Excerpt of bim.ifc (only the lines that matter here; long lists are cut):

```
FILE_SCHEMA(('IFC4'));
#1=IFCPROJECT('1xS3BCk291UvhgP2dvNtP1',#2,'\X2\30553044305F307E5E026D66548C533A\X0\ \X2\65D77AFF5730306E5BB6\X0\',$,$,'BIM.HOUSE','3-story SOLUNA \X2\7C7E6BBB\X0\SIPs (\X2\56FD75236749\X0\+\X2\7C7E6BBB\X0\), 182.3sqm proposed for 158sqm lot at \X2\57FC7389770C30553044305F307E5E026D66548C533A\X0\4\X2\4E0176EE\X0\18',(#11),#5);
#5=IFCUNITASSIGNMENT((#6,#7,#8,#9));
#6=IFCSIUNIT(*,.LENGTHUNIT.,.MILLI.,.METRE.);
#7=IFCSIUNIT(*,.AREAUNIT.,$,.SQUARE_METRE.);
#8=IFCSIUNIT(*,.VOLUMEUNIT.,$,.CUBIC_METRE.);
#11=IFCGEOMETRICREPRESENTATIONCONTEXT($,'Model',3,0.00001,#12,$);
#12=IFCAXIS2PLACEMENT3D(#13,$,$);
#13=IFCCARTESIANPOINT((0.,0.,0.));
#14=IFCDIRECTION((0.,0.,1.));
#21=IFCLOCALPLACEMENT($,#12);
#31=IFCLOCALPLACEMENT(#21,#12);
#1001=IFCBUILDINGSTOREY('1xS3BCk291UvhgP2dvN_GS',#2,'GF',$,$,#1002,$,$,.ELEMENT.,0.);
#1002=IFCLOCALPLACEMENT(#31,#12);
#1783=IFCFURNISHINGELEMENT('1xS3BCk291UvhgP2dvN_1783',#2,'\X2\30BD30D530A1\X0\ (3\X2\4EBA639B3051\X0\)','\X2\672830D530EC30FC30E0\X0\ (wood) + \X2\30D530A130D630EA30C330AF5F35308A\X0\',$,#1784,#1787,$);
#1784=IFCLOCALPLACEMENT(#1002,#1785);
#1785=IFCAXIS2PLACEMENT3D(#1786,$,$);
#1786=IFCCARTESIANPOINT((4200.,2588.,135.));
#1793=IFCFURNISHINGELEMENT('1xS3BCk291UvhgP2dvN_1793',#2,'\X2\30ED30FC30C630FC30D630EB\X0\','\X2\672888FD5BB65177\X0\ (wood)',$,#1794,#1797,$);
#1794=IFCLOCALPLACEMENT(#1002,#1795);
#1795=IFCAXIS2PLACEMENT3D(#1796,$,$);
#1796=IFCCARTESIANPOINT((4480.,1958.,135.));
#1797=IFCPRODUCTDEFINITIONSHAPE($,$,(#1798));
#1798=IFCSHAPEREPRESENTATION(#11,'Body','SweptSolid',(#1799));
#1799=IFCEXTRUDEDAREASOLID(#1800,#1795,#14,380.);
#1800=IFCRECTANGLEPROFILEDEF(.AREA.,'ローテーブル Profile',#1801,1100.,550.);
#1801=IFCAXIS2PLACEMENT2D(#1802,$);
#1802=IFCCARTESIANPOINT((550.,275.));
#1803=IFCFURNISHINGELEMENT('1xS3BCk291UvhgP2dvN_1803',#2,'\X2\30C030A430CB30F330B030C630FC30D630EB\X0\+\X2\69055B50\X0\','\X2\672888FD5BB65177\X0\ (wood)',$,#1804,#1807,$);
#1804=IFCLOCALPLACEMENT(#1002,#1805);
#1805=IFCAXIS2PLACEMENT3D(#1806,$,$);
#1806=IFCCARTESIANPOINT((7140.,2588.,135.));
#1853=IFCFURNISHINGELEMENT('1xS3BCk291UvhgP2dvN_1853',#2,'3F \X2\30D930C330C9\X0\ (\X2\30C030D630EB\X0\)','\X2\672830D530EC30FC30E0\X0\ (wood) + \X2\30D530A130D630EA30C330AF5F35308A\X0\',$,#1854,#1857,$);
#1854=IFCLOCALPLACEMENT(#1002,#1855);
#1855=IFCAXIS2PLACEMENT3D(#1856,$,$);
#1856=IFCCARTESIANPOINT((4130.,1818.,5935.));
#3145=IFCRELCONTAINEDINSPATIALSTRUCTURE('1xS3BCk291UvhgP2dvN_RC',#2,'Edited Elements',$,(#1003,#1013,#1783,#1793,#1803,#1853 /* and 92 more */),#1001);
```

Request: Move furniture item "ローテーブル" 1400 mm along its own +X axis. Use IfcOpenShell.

```python
import ifcopenshell
import ifcopenshell.api.geometry
import ifcopenshell.util.placement

model = ifcopenshell.open("bim.ifc")

item = model.by_guid("1xS3BCk291UvhgP2dvN_1793")
matrix = ifcopenshell.util.placement.get_local_placement(item.ObjectPlacement)
matrix[:3, 3] += matrix[:3, 0] * 1400.0
ifcopenshell.api.geometry.edit_object_placement(model, product=item, matrix=matrix, is_si=False)

print(ifcopenshell.util.placement.get_local_placement(item.ObjectPlacement).round(3) + 0.0)

model.write("bim-out.ifc")
```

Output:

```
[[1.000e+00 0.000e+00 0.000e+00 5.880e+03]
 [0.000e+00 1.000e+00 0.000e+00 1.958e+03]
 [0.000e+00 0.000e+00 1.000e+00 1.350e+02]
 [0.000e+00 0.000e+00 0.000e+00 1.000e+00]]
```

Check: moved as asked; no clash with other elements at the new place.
